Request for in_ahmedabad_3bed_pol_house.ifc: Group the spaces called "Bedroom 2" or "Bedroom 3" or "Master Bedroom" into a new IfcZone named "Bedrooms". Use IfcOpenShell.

First a look at what the model holds.

```python
import ifcopenshell

model = ifcopenshell.open("in_ahmedabad_3bed_pol_house.ifc")
print(model.schema)
seen = {}
for space in model.by_type("IfcSpace"):
    seen[space.LongName] = seen.get(space.LongName, 0) + 1
for name, count in sorted(seen.items(), key=str):
    print(count, "x", name)
print("zones:", [z.Name for z in model.by_type("IfcZone")][:20])
```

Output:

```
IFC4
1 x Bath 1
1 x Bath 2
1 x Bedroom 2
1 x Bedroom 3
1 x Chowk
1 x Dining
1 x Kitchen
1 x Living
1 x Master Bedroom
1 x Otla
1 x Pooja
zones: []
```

```python
import ifcopenshell
import ifcopenshell.api.group
import ifcopenshell.api.root

model = ifcopenshell.open("in_ahmedabad_3bed_pol_house.ifc")

names = {"Bedroom 2", "Bedroom 3", "Master Bedroom"}
spaces = [s for s in model.by_type("IfcSpace") if s.LongName in names]

zone = ifcopenshell.api.root.create_entity(model, ifc_class="IfcZone", name="Bedrooms")
ifcopenshell.api.group.assign_group(model, products=spaces, group=zone)
print(len(spaces), "spaces in", zone.Name)

model.write("in_ahmedabad_3bed_pol_house_edited.ifc")
```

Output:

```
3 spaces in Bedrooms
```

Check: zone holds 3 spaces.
